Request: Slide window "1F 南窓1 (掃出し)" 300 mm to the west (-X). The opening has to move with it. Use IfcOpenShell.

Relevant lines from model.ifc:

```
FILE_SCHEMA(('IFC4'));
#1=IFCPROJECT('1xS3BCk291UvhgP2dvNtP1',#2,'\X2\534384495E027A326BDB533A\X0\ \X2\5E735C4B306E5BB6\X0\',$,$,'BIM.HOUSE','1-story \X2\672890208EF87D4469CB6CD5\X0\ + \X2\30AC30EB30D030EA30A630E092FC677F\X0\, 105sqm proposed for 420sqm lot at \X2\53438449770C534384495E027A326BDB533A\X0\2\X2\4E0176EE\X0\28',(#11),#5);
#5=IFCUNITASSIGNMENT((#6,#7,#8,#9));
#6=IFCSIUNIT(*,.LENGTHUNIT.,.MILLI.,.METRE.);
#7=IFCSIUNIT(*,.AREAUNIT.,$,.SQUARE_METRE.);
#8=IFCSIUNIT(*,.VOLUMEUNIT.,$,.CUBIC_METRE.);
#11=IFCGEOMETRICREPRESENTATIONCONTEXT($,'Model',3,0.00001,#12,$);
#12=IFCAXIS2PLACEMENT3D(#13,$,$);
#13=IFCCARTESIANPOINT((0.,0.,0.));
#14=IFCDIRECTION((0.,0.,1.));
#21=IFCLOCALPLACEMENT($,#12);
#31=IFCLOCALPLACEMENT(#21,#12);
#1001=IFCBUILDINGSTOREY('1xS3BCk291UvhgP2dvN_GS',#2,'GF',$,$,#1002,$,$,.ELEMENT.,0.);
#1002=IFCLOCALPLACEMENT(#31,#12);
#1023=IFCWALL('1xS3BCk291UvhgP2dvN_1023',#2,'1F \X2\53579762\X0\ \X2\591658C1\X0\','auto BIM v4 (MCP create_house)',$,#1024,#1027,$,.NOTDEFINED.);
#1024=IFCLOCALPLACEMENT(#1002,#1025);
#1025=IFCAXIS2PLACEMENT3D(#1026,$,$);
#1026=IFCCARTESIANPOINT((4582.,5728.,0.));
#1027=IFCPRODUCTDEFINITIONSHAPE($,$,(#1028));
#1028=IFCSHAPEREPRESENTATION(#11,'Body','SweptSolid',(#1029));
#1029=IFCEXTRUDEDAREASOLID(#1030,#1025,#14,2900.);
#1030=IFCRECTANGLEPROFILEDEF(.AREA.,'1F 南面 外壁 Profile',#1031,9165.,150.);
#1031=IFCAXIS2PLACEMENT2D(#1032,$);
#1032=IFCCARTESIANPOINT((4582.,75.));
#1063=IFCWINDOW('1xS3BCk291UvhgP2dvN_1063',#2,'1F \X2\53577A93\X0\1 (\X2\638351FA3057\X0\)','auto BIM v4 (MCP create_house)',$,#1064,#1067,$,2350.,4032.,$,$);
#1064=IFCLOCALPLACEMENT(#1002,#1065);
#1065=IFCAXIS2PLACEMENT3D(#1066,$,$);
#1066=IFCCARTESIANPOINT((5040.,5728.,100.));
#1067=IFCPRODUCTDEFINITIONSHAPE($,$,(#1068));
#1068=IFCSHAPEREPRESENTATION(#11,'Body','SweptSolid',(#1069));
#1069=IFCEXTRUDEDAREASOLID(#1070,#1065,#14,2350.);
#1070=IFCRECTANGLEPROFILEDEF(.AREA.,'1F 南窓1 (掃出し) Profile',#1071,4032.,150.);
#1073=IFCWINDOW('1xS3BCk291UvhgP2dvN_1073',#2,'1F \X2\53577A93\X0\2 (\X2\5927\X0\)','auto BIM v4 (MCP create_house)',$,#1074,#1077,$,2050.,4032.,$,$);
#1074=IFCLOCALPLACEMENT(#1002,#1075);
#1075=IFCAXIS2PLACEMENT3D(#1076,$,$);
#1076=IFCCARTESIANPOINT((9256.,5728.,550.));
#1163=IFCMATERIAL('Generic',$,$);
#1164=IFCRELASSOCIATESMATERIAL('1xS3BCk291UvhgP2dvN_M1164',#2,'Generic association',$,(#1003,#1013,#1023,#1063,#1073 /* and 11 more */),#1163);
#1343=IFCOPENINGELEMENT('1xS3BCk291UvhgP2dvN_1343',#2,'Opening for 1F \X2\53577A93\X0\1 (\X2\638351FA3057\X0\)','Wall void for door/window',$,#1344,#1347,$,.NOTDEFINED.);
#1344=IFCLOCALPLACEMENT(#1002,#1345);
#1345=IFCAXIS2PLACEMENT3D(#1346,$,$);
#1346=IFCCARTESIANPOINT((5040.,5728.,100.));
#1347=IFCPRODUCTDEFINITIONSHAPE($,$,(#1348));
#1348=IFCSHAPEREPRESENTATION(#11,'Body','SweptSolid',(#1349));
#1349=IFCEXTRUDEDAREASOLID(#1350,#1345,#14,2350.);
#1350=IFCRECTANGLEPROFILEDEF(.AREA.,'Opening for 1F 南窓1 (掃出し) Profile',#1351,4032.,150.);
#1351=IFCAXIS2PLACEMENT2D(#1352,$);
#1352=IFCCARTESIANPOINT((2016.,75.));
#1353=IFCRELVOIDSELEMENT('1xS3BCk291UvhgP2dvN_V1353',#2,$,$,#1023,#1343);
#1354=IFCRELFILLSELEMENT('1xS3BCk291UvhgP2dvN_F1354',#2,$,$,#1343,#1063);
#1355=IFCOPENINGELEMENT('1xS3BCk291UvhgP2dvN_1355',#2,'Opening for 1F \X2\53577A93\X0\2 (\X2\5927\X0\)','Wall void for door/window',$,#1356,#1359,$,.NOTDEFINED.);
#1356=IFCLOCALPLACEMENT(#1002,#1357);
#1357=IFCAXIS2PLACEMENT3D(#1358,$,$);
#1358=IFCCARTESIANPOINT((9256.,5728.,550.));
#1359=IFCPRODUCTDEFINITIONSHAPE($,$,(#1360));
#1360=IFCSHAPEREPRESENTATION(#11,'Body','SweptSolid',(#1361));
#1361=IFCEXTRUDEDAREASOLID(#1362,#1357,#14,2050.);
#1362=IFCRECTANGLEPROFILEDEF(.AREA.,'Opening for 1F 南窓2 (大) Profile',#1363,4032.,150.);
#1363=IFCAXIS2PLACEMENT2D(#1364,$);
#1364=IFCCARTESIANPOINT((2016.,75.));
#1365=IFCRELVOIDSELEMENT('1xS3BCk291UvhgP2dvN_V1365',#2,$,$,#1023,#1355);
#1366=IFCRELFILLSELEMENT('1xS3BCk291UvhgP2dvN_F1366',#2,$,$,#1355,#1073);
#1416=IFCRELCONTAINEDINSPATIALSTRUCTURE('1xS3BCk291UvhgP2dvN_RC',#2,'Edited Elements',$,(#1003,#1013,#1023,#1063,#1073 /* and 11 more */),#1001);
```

```python
import ifcopenshell
import ifcopenshell.api.geometry
import ifcopenshell.util.placement
import ifcopenshell.util.unit

model = ifcopenshell.open("model.ifc")
unit_scale = ifcopenshell.util.unit.calculate_unit_scale(model)

window = model.by_guid("1xS3BCk291UvhgP2dvN_1063")
opening = window.FillsVoids[0].RelatingOpeningElement
wall = opening.VoidsElements[0].RelatingBuildingElement

wall_matrix = ifcopenshell.util.placement.get_local_placement(wall.ObjectPlacement)
shift = wall_matrix[:3, 0] * -0.3 / unit_scale
before = ifcopenshell.util.placement.get_local_placement(window.ObjectPlacement)[:3, 3].copy()

# The window is not placed relative to its opening, so move both.
for product in (opening, window):
    matrix = ifcopenshell.util.placement.get_local_placement(product.ObjectPlacement)
    matrix[:3, 3] += shift
    ifcopenshell.api.geometry.edit_object_placement(model, product=product, matrix=matrix, is_si=False)

after = ifcopenshell.util.placement.get_local_placement(window.ObjectPlacement)[:3, 3]
print("window moved by", (after - before).round(3) + 0.0)

model.write("model_v2.ifc")
```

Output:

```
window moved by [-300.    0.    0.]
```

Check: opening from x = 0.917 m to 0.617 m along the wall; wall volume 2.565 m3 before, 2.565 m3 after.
